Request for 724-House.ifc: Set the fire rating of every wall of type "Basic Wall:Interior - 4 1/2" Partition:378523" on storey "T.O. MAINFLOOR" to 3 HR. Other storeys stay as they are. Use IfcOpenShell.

First a look at what the model holds.

```python
import ifcopenshell
import ifcopenshell.util.element

model = ifcopenshell.open("724-House.ifc")
print(model.schema)
storey = next(s for s in model.by_type("IfcBuildingStorey") if s.Name == "T.O. MAINFLOOR")
walls = [e for e in ifcopenshell.util.element.get_decomposition(storey) if e.is_a("IfcWall")]
seen = {}
for e in walls:
    element_type = ifcopenshell.util.element.get_type(e)
    key = (element_type.Name if element_type != e and element_type else None, ifcopenshell.util.element.get_pset(e, "Pset_WallCommon", "FireRating"))
    seen[key] = seen.get(key, 0) + 1
for (name, value), count in sorted(seen.items(), key=str):
    print(count, "x", name, "|", value)
```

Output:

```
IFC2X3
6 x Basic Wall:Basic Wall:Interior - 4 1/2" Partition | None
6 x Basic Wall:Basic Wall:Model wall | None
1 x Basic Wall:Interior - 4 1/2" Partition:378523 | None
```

```python
import ifcopenshell
import ifcopenshell.api.pset
import ifcopenshell.util.element

model = ifcopenshell.open("724-House.ifc")

storey = next(s for s in model.by_type("IfcBuildingStorey") if s.Name == "T.O. MAINFLOOR")
walls = [e for e in ifcopenshell.util.element.get_decomposition(storey) if e.is_a("IfcWall")]

count = 0
for e in walls:
    element_type = ifcopenshell.util.element.get_type(e)
    if element_type in (None, e) or element_type.Name != 'Basic Wall:Interior - 4 1/2" Partition:378523':
        continue
    # add_pset returns the element's existing set when there is one.
    pset = ifcopenshell.api.pset.add_pset(model, product=e, name="Pset_WallCommon")
    ifcopenshell.api.pset.edit_pset(model, pset=pset, properties={"FireRating": "3 HR"})
    count += 1

print(count, "walls updated")

model.write("724-House_rev.ifc")
```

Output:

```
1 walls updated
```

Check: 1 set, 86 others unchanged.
